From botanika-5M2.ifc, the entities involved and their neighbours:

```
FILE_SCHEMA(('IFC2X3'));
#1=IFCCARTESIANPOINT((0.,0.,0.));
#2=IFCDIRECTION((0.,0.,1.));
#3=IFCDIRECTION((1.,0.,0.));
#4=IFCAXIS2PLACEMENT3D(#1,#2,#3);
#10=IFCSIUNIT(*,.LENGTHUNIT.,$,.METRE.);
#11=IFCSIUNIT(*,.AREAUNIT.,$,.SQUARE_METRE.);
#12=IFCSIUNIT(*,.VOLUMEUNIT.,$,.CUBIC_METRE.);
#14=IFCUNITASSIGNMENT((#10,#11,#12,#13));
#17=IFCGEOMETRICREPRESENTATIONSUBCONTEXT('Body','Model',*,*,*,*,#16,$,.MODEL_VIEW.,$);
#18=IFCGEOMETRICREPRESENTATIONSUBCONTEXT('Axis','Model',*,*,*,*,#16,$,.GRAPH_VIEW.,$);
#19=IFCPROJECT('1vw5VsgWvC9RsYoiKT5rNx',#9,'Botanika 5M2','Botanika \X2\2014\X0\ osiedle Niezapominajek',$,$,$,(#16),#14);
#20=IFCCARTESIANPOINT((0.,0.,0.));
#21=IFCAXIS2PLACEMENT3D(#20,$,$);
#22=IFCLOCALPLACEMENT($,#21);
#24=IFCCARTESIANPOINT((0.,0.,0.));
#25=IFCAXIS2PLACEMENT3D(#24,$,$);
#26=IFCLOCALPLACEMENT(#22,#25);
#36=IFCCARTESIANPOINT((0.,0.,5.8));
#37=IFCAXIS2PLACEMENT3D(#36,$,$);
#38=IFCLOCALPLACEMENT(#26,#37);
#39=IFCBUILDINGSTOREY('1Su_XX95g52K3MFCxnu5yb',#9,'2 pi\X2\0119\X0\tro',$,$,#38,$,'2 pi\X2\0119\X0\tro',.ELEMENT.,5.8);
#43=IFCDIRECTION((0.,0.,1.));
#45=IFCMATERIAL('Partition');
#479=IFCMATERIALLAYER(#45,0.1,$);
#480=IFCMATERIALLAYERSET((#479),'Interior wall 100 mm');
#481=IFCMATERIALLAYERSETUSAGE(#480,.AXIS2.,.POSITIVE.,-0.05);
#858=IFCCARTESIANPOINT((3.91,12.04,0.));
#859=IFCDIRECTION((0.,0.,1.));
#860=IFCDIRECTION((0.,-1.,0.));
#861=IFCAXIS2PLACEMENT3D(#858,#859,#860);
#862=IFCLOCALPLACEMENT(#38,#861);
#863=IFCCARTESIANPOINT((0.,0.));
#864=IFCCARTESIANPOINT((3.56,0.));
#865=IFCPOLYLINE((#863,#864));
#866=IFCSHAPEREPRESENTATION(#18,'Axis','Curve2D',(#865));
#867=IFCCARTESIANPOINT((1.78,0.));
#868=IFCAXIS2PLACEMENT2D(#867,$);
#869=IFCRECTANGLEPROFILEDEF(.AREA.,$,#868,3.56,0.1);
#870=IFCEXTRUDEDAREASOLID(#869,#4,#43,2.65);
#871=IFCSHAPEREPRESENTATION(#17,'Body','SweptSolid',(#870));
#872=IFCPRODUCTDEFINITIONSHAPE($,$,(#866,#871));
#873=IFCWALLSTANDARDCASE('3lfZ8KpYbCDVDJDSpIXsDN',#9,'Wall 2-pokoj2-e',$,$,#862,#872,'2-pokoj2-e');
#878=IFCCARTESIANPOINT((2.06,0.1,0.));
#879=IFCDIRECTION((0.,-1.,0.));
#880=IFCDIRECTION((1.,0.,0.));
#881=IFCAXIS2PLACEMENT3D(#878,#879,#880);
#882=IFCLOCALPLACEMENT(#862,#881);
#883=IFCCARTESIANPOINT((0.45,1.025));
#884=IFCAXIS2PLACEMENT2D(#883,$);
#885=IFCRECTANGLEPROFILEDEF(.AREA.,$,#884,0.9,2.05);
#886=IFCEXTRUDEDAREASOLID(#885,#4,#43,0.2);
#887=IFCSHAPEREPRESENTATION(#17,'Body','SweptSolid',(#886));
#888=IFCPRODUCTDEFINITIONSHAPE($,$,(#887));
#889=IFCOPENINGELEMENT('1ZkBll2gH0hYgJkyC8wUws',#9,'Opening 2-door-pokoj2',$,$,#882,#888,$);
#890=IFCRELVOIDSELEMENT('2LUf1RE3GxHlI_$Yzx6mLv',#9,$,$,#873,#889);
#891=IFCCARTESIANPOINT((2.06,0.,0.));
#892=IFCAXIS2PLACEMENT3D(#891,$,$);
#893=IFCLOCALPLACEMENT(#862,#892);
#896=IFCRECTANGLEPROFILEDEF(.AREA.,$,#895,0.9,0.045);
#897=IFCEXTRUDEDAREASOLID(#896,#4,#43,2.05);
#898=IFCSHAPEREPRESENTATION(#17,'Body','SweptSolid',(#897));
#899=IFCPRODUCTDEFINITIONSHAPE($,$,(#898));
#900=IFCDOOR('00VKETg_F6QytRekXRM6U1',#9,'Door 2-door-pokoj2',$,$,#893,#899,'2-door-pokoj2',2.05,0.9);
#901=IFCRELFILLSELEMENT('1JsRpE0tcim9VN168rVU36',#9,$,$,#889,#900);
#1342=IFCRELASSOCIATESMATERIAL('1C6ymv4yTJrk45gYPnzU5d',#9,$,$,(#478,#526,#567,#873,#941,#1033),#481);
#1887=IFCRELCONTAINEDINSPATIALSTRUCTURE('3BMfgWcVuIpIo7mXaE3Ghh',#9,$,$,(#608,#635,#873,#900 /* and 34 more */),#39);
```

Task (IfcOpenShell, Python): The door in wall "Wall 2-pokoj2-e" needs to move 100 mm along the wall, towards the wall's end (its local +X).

```python
import ifcopenshell
import ifcopenshell.api.geometry
import ifcopenshell.util.placement
import ifcopenshell.util.unit

model = ifcopenshell.open("botanika-5M2.ifc")
unit_scale = ifcopenshell.util.unit.calculate_unit_scale(model)

door = model.by_id(900)
opening = door.FillsVoids[0].RelatingOpeningElement
wall = opening.VoidsElements[0].RelatingBuildingElement

wall_matrix = ifcopenshell.util.placement.get_local_placement(wall.ObjectPlacement)
shift = wall_matrix[:3, 0] * 0.1 / unit_scale
before = ifcopenshell.util.placement.get_local_placement(door.ObjectPlacement)[:3, 3].copy()

# The door is not placed relative to its opening, so move both.
for product in (opening, door):
    matrix = ifcopenshell.util.placement.get_local_placement(product.ObjectPlacement)
    matrix[:3, 3] += shift
    ifcopenshell.api.geometry.edit_object_placement(model, product=product, matrix=matrix, is_si=False)

after = ifcopenshell.util.placement.get_local_placement(door.ObjectPlacement)[:3, 3]
print("door moved by", (after - before).round(3) + 0.0)

model.write("botanika-5M2-out.ifc")
```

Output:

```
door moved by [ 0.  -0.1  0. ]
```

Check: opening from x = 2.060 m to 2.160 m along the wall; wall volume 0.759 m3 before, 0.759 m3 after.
